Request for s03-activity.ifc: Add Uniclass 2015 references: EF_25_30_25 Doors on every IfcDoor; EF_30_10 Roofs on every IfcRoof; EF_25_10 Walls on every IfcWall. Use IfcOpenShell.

First a look at what the model holds.

```python
import ifcopenshell

model = ifcopenshell.open("s03-activity.ifc")
print(model.schema)
print("classifications:", [c.Name for c in model.by_type("IfcClassification")])
for ifc_class in ("IfcDoor", "IfcRoof", "IfcStair", "IfcWall", "IfcWindow"):
    print(ifc_class, len(model.by_type(ifc_class)))
```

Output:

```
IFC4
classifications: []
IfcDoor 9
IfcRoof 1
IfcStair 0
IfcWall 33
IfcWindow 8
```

```python
import ifcopenshell
import ifcopenshell.api.classification

model = ifcopenshell.open("s03-activity.ifc")

system = ifcopenshell.api.classification.add_classification(model, classification="Uniclass 2015")

codes = {
    "IfcDoor": ("EF_25_30_25", "Doors"),
    "IfcRoof": ("EF_30_10", "Roofs"),
    "IfcWall": ("EF_25_10", "Walls"),
}
for ifc_class, (code, name) in codes.items():
    products = model.by_type(ifc_class)
    ifcopenshell.api.classification.add_reference(
        model, products=products, classification=system, identification=code, name=name
    )
    print(code, len(products))

model.write("s03-activity-out.ifc")
```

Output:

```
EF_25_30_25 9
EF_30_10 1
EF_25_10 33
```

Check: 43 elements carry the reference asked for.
